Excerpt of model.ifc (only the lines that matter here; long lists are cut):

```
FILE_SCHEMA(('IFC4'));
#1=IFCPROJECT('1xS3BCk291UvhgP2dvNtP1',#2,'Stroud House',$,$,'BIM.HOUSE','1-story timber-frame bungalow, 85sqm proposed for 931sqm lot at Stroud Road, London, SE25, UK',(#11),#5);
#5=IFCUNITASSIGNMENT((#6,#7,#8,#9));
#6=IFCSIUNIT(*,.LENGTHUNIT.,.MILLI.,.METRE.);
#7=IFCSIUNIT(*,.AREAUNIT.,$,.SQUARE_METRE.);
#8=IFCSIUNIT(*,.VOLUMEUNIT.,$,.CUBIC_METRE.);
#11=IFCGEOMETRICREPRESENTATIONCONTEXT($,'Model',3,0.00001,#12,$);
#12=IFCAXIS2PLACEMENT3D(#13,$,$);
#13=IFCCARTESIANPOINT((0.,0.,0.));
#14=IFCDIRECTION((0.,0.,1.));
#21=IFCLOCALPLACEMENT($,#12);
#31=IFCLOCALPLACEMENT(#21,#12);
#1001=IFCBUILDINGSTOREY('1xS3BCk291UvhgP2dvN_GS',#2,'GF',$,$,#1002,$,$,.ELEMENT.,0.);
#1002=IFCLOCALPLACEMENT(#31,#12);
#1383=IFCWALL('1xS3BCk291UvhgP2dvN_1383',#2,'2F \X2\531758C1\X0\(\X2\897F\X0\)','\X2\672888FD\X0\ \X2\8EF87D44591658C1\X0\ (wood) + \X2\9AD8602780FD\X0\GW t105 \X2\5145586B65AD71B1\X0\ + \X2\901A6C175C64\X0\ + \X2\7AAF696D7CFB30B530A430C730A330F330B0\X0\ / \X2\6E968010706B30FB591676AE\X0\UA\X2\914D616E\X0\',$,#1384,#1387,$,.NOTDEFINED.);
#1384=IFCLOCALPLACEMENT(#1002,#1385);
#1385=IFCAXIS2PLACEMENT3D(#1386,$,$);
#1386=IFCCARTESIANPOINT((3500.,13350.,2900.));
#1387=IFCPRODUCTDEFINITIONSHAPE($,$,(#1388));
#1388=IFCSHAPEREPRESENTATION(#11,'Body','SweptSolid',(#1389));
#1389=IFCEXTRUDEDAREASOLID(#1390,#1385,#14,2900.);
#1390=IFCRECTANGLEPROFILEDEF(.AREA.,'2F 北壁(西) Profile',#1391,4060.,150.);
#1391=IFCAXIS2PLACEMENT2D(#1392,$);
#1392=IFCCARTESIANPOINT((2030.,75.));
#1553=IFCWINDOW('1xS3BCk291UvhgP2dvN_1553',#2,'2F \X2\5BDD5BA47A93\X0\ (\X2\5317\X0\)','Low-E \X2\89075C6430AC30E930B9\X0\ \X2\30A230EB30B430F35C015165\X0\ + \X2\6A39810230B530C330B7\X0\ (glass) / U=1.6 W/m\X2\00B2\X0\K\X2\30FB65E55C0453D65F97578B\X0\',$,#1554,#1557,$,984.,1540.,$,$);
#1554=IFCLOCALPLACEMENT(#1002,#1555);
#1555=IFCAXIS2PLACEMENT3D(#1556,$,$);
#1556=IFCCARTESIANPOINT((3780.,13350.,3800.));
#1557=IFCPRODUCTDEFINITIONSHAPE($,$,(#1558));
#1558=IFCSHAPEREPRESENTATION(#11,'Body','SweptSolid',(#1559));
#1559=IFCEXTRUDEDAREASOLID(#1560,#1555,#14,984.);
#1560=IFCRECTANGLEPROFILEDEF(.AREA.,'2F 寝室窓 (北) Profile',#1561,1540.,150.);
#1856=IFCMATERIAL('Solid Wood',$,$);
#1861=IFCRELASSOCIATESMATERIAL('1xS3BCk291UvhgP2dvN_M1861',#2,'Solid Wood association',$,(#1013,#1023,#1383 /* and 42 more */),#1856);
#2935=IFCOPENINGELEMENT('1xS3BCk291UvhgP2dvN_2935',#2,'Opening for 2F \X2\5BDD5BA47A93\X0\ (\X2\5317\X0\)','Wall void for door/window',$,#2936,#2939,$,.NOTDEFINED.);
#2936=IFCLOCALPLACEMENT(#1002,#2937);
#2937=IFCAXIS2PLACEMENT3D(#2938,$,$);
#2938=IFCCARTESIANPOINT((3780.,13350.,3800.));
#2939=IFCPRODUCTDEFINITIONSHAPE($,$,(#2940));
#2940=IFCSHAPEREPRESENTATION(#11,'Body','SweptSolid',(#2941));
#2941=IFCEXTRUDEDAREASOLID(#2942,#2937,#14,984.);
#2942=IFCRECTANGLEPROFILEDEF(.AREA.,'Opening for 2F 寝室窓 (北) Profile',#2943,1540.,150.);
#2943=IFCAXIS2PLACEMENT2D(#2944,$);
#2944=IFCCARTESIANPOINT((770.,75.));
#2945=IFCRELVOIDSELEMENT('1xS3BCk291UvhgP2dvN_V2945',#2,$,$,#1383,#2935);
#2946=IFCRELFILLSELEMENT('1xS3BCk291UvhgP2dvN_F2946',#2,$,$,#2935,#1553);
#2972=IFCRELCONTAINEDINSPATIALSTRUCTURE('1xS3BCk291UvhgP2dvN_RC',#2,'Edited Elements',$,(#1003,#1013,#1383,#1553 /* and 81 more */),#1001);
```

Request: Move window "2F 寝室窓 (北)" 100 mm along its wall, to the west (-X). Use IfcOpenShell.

```python
import ifcopenshell
import ifcopenshell.api.geometry
import ifcopenshell.util.placement

model = ifcopenshell.open("model.ifc")

window = model.by_guid("1xS3BCk291UvhgP2dvN_1553")
opening = window.FillsVoids[0].RelatingOpeningElement
wall = opening.VoidsElements[0].RelatingBuildingElement

wall_matrix = ifcopenshell.util.placement.get_local_placement(wall.ObjectPlacement)
shift = wall_matrix[:3, 0] * -100.0
before = ifcopenshell.util.placement.get_local_placement(window.ObjectPlacement)[:3, 3].copy()

# The window is not placed relative to its opening, so move both.
for product in (opening, window):
    matrix = ifcopenshell.util.placement.get_local_placement(product.ObjectPlacement)
    matrix[:3, 3] += shift
    ifcopenshell.api.geometry.edit_object_placement(model, product=product, matrix=matrix, is_si=False)

after = ifcopenshell.util.placement.get_local_placement(window.ObjectPlacement)[:3, 3]
print("window moved by", (after - before).round(3) + 0.0)

model.write("model_v2.ifc")
```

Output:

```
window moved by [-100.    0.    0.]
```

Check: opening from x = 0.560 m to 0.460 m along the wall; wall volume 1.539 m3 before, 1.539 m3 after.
